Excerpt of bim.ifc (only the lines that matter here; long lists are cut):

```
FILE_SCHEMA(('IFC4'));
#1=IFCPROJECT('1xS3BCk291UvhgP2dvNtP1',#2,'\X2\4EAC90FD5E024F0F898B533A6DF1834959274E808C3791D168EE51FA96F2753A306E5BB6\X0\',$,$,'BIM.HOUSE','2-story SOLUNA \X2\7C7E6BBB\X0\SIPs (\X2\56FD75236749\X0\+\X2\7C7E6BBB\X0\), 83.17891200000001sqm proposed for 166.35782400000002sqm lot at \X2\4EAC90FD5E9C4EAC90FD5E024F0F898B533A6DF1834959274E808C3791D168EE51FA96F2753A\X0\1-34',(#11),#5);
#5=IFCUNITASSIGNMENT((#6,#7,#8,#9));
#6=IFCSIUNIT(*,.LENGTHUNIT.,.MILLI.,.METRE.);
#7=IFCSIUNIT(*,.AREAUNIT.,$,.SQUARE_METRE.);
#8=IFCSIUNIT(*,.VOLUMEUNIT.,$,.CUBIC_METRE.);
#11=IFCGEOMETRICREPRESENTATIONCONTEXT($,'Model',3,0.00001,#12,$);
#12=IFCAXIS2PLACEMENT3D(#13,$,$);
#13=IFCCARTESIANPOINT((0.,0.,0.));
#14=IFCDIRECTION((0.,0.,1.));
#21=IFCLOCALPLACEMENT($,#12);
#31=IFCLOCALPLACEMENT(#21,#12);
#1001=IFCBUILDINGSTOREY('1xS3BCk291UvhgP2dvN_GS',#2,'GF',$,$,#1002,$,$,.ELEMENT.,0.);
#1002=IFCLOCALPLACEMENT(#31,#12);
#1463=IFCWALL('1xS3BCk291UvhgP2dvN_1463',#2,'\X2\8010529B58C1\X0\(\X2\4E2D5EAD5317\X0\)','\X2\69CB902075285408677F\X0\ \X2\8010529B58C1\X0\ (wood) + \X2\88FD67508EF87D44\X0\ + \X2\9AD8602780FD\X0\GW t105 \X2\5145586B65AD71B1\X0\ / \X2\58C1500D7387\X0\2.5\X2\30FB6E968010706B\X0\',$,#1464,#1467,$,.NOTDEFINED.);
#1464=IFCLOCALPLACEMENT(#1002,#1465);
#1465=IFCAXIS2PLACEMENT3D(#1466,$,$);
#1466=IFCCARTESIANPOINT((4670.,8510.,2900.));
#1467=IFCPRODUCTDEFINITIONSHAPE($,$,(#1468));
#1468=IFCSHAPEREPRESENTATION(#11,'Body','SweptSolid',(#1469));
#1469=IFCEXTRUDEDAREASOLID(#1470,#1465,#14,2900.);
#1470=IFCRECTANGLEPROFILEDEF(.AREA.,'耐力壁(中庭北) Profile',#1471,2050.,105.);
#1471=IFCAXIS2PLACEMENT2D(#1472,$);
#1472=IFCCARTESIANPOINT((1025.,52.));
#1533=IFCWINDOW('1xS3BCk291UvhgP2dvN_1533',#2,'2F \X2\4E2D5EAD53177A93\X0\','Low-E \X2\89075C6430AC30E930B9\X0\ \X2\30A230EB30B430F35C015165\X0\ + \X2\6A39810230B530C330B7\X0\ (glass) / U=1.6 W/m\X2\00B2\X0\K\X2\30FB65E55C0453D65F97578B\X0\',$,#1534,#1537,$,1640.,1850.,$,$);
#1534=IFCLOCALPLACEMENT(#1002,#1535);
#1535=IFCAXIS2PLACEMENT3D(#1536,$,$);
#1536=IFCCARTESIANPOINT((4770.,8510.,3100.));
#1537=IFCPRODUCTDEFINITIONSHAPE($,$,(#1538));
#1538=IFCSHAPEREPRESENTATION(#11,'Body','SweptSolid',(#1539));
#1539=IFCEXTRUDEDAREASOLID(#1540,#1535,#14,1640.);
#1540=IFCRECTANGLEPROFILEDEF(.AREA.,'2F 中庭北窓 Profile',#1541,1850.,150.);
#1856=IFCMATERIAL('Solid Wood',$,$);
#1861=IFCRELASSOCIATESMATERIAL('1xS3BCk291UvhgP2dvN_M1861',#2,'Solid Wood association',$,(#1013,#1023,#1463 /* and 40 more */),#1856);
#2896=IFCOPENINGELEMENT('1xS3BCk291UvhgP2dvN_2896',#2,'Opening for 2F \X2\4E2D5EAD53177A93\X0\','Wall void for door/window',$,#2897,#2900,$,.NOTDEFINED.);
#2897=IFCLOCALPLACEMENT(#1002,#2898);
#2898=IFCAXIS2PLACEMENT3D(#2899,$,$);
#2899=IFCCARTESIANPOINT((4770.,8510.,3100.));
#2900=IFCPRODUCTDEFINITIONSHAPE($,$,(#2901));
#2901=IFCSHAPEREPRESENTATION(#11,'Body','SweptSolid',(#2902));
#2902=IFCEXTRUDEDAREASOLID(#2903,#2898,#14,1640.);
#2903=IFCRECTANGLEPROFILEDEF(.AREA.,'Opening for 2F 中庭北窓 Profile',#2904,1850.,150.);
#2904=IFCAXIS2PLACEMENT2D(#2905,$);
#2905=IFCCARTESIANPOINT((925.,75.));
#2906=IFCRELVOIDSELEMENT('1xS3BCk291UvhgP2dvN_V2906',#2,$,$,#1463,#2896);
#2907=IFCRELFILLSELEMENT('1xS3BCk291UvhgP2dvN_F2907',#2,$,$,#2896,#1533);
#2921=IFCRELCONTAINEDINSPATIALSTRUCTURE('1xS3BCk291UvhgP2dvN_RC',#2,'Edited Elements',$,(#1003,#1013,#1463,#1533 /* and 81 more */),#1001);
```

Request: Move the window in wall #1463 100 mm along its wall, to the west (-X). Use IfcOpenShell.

```python
import ifcopenshell
import ifcopenshell.api.geometry
import ifcopenshell.util.placement
import ifcopenshell.util.unit

model = ifcopenshell.open("bim.ifc")
unit_scale = ifcopenshell.util.unit.calculate_unit_scale(model)

window = model.by_guid("1xS3BCk291UvhgP2dvN_1533")
opening = window.FillsVoids[0].RelatingOpeningElement
wall = opening.VoidsElements[0].RelatingBuildingElement

wall_matrix = ifcopenshell.util.placement.get_local_placement(wall.ObjectPlacement)
shift = wall_matrix[:3, 0] * -0.1 / unit_scale
before = ifcopenshell.util.placement.get_local_placement(window.ObjectPlacement)[:3, 3].copy()

# The window is not placed relative to its opening, so move both.
for product in (opening, window):
    matrix = ifcopenshell.util.placement.get_local_placement(product.ObjectPlacement)
    matrix[:3, 3] += shift
    ifcopenshell.api.geometry.edit_object_placement(model, product=product, matrix=matrix, is_si=False)

after = ifcopenshell.util.placement.get_local_placement(window.ObjectPlacement)[:3, 3]
print("window moved by", (after - before).round(3) + 0.0)

model.write("bim_edited.ifc")
```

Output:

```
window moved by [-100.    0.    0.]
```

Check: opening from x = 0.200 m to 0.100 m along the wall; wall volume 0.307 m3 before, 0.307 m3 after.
